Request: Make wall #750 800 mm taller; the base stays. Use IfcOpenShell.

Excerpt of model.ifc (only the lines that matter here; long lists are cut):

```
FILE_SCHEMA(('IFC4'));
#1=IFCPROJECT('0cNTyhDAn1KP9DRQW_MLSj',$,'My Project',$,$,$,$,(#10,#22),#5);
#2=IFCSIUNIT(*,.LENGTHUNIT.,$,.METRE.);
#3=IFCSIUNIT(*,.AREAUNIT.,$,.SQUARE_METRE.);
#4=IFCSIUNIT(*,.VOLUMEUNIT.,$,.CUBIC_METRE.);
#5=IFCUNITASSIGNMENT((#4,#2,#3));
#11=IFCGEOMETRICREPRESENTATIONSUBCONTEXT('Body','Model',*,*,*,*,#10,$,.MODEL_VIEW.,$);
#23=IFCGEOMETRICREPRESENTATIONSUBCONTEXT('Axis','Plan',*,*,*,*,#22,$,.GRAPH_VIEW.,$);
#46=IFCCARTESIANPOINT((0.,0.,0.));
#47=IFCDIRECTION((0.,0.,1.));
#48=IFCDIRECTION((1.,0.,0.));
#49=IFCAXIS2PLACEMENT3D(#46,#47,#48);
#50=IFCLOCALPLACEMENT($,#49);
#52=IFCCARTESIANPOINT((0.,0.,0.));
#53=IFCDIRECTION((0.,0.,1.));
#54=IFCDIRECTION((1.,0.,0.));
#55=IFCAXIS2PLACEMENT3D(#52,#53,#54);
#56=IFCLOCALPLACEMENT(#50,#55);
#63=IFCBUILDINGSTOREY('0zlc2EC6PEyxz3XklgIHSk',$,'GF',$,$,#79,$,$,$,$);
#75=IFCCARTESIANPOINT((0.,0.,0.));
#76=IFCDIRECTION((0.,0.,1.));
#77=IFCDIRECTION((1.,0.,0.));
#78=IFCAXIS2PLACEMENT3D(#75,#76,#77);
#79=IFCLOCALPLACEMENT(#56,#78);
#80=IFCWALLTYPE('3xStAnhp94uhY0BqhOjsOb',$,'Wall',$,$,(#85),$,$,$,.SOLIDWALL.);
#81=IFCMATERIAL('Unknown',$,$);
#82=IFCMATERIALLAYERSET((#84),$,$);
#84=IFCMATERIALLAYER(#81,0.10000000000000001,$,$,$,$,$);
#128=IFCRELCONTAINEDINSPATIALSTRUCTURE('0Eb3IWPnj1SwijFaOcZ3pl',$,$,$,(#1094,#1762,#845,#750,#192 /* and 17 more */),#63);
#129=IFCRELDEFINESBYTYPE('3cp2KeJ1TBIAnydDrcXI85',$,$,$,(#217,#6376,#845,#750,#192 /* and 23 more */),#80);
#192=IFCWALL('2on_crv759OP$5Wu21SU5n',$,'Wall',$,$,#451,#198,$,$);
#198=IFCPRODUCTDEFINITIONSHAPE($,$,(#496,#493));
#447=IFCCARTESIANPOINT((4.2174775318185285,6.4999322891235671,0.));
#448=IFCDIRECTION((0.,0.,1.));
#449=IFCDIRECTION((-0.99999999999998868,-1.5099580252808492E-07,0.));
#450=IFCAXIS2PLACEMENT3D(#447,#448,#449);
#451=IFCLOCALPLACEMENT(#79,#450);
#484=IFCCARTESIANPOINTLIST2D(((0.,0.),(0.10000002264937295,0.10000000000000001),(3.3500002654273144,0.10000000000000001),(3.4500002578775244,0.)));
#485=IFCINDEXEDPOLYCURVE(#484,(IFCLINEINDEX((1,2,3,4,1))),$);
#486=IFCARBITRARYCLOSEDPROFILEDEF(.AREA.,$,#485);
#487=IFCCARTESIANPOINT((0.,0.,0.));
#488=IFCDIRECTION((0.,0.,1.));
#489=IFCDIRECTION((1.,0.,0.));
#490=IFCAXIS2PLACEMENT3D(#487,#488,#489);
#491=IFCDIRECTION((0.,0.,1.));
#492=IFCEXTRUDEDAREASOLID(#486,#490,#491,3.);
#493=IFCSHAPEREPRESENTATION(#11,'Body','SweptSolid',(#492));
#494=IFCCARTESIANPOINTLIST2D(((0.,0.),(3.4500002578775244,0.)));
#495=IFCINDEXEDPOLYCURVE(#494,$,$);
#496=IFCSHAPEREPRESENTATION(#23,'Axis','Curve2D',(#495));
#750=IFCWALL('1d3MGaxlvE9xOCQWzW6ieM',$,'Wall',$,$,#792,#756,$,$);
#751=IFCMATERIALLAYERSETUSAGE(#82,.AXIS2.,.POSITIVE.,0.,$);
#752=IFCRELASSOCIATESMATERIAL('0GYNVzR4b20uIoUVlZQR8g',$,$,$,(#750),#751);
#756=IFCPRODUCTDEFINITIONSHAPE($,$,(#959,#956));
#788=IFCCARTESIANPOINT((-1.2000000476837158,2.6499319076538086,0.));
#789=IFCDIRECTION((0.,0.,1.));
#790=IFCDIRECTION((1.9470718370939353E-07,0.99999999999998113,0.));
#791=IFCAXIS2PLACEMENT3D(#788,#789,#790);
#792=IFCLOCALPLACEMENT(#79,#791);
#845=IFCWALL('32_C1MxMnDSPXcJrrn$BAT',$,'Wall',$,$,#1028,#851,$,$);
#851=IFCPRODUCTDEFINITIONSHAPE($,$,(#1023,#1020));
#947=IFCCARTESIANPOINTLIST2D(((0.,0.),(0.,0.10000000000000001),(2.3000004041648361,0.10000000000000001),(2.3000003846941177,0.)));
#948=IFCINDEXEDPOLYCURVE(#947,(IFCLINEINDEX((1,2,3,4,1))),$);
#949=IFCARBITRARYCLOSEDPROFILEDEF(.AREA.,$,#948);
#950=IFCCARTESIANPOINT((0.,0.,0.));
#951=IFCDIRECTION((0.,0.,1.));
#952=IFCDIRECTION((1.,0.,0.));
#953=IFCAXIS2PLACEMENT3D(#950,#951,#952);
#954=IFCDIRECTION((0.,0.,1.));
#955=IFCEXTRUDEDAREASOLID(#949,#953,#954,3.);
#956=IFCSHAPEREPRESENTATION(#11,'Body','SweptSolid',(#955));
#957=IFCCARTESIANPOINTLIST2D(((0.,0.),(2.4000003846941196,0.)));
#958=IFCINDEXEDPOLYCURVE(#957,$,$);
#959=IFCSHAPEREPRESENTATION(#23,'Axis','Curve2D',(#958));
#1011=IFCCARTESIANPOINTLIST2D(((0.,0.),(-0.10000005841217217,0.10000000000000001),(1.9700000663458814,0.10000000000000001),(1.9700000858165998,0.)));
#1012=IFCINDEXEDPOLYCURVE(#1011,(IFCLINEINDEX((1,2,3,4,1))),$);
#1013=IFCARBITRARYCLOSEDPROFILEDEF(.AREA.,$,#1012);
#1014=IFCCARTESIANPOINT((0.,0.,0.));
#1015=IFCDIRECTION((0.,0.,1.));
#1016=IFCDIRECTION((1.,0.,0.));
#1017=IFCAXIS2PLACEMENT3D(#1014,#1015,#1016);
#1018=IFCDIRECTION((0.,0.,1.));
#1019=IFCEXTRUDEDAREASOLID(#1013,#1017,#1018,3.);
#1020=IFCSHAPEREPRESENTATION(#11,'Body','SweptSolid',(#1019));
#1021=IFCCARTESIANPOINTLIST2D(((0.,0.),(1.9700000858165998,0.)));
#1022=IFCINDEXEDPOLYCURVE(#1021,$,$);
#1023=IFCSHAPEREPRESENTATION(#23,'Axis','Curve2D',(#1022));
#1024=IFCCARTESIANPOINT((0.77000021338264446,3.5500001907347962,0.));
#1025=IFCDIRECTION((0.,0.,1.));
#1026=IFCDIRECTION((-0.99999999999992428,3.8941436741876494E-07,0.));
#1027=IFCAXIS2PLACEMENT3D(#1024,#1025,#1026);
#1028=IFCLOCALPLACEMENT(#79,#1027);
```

```python
import ifcopenshell
import ifcopenshell.geom
import ifcopenshell.util.representation
import ifcopenshell.util.shape
import ifcopenshell.util.unit

model = ifcopenshell.open("model.ifc")
unit_scale = ifcopenshell.util.unit.calculate_unit_scale(model)
settings = ifcopenshell.geom.settings()


def volume(element):
    """Net volume in cubic metres, openings subtracted."""
    shape = ifcopenshell.geom.create_shape(settings, element)
    return ifcopenshell.util.shape.get_volume(shape.geometry)


wall = model.by_guid("1d3MGaxlvE9xOCQWzW6ieM")
before = volume(wall)

body = ifcopenshell.util.representation.get_representation(wall, "Model", "Body")
solid = body.Items[0]
old_height = solid.Depth
solid.Depth += 0.8 / unit_scale
after = volume(wall)

print(f"height {old_height:g} -> {solid.Depth:g}, volume {before:.3f} -> {after:.3f} m3")

model.write("model-out.ifc")
```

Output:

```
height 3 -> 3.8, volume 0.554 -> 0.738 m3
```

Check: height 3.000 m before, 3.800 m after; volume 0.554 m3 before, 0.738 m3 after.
